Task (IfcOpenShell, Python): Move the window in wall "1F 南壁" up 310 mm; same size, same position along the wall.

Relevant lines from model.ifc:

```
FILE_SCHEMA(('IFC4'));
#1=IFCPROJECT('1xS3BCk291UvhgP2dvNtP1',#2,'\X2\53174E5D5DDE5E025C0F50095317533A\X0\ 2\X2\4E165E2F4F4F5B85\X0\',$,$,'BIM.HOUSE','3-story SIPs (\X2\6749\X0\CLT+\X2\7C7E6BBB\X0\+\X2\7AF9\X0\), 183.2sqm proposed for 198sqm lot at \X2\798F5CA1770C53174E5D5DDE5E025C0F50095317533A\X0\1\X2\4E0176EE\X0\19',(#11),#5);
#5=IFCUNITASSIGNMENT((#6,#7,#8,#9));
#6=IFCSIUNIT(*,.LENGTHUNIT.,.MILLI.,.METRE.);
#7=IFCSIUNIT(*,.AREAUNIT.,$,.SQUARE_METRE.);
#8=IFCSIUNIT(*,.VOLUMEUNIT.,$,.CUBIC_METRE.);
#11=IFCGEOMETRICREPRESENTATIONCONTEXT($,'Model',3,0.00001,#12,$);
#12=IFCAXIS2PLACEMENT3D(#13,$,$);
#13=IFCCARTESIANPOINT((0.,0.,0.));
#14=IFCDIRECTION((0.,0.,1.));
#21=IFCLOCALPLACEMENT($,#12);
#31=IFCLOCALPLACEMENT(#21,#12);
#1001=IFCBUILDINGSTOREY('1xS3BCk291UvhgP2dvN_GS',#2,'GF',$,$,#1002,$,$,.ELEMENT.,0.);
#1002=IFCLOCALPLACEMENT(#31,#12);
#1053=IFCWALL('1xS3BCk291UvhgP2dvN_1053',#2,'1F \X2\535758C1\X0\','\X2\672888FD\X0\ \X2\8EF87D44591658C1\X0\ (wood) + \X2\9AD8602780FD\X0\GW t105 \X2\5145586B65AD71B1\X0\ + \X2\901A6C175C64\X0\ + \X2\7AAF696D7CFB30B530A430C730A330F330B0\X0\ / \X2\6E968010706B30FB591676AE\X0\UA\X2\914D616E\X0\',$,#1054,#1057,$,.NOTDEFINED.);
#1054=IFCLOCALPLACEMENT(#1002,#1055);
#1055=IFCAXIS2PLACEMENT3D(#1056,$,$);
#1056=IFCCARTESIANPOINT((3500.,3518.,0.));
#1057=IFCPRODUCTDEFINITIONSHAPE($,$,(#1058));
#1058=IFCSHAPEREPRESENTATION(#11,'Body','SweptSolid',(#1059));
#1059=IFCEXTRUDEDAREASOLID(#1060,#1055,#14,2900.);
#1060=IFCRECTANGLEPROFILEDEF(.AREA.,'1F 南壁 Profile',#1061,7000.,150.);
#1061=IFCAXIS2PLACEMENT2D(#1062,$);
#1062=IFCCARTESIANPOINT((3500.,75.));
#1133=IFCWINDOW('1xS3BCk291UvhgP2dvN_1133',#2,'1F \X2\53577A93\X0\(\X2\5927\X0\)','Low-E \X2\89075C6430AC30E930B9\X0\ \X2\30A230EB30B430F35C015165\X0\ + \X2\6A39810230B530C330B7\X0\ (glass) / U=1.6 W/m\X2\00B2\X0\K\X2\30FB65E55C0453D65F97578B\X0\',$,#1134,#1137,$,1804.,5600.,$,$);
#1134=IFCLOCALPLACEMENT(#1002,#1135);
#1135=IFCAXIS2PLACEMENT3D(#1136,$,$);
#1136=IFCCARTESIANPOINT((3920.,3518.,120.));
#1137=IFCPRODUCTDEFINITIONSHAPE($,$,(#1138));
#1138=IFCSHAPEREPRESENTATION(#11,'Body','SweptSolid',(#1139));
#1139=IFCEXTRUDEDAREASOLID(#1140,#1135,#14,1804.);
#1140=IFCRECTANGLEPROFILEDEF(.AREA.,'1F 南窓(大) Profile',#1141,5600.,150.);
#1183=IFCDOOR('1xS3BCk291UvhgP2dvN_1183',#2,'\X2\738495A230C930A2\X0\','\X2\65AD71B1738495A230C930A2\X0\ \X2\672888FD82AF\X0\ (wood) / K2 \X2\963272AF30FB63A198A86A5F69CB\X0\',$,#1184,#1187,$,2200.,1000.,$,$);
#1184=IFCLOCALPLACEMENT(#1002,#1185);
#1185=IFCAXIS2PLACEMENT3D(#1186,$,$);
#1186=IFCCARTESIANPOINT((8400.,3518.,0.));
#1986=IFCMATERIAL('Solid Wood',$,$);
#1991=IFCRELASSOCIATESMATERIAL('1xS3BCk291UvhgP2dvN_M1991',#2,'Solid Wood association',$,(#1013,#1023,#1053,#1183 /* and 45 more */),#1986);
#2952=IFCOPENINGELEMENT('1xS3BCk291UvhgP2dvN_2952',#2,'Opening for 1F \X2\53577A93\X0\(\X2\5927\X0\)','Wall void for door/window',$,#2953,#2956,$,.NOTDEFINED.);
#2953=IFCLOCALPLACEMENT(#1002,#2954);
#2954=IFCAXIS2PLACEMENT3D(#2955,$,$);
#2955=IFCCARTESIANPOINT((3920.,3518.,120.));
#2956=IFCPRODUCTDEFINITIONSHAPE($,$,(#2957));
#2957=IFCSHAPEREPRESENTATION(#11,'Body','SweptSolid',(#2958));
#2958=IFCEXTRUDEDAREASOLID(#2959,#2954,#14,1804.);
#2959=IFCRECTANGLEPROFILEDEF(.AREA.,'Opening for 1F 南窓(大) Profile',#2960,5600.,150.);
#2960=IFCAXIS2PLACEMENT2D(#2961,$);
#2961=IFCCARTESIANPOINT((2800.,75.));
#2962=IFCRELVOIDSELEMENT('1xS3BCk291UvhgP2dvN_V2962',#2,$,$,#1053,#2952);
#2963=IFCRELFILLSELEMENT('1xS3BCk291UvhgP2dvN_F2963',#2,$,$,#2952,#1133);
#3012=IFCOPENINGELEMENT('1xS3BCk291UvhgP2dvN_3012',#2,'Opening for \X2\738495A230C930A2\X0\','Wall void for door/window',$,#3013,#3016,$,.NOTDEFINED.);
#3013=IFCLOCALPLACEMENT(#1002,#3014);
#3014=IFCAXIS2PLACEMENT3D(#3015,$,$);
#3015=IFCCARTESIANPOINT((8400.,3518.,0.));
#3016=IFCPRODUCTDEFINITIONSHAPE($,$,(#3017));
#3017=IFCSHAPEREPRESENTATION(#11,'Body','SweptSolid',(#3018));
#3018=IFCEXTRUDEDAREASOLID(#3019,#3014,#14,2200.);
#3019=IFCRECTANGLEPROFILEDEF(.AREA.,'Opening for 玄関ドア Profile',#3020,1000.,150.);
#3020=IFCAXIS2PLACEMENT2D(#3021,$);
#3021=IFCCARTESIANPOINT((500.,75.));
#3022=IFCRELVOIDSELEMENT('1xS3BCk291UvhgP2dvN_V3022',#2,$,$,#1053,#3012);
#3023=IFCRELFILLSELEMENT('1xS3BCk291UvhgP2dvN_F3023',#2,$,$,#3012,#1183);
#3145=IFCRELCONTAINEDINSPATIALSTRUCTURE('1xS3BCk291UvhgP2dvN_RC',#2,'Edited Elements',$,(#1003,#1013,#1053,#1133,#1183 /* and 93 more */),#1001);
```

```python
import numpy as np
import ifcopenshell
import ifcopenshell.api.geometry
import ifcopenshell.util.placement
import ifcopenshell.util.unit

model = ifcopenshell.open("model.ifc")
unit_scale = ifcopenshell.util.unit.calculate_unit_scale(model)

window = model.by_guid("1xS3BCk291UvhgP2dvN_1133")
opening = window.FillsVoids[0].RelatingOpeningElement
dz = 310.0

shift = np.array([0.0, 0.0, dz])
# The window is not placed relative to its opening, so move both.
for product in (opening, window):
    matrix = ifcopenshell.util.placement.get_local_placement(product.ObjectPlacement)
    matrix[:3, 3] += shift
    ifcopenshell.api.geometry.edit_object_placement(model, product=product, matrix=matrix, is_si=False)

print(f"moved by {dz * unit_scale:+.3f} m")

model.write("model_v2.ifc")
```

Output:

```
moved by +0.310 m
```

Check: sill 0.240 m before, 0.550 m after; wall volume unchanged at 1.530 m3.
